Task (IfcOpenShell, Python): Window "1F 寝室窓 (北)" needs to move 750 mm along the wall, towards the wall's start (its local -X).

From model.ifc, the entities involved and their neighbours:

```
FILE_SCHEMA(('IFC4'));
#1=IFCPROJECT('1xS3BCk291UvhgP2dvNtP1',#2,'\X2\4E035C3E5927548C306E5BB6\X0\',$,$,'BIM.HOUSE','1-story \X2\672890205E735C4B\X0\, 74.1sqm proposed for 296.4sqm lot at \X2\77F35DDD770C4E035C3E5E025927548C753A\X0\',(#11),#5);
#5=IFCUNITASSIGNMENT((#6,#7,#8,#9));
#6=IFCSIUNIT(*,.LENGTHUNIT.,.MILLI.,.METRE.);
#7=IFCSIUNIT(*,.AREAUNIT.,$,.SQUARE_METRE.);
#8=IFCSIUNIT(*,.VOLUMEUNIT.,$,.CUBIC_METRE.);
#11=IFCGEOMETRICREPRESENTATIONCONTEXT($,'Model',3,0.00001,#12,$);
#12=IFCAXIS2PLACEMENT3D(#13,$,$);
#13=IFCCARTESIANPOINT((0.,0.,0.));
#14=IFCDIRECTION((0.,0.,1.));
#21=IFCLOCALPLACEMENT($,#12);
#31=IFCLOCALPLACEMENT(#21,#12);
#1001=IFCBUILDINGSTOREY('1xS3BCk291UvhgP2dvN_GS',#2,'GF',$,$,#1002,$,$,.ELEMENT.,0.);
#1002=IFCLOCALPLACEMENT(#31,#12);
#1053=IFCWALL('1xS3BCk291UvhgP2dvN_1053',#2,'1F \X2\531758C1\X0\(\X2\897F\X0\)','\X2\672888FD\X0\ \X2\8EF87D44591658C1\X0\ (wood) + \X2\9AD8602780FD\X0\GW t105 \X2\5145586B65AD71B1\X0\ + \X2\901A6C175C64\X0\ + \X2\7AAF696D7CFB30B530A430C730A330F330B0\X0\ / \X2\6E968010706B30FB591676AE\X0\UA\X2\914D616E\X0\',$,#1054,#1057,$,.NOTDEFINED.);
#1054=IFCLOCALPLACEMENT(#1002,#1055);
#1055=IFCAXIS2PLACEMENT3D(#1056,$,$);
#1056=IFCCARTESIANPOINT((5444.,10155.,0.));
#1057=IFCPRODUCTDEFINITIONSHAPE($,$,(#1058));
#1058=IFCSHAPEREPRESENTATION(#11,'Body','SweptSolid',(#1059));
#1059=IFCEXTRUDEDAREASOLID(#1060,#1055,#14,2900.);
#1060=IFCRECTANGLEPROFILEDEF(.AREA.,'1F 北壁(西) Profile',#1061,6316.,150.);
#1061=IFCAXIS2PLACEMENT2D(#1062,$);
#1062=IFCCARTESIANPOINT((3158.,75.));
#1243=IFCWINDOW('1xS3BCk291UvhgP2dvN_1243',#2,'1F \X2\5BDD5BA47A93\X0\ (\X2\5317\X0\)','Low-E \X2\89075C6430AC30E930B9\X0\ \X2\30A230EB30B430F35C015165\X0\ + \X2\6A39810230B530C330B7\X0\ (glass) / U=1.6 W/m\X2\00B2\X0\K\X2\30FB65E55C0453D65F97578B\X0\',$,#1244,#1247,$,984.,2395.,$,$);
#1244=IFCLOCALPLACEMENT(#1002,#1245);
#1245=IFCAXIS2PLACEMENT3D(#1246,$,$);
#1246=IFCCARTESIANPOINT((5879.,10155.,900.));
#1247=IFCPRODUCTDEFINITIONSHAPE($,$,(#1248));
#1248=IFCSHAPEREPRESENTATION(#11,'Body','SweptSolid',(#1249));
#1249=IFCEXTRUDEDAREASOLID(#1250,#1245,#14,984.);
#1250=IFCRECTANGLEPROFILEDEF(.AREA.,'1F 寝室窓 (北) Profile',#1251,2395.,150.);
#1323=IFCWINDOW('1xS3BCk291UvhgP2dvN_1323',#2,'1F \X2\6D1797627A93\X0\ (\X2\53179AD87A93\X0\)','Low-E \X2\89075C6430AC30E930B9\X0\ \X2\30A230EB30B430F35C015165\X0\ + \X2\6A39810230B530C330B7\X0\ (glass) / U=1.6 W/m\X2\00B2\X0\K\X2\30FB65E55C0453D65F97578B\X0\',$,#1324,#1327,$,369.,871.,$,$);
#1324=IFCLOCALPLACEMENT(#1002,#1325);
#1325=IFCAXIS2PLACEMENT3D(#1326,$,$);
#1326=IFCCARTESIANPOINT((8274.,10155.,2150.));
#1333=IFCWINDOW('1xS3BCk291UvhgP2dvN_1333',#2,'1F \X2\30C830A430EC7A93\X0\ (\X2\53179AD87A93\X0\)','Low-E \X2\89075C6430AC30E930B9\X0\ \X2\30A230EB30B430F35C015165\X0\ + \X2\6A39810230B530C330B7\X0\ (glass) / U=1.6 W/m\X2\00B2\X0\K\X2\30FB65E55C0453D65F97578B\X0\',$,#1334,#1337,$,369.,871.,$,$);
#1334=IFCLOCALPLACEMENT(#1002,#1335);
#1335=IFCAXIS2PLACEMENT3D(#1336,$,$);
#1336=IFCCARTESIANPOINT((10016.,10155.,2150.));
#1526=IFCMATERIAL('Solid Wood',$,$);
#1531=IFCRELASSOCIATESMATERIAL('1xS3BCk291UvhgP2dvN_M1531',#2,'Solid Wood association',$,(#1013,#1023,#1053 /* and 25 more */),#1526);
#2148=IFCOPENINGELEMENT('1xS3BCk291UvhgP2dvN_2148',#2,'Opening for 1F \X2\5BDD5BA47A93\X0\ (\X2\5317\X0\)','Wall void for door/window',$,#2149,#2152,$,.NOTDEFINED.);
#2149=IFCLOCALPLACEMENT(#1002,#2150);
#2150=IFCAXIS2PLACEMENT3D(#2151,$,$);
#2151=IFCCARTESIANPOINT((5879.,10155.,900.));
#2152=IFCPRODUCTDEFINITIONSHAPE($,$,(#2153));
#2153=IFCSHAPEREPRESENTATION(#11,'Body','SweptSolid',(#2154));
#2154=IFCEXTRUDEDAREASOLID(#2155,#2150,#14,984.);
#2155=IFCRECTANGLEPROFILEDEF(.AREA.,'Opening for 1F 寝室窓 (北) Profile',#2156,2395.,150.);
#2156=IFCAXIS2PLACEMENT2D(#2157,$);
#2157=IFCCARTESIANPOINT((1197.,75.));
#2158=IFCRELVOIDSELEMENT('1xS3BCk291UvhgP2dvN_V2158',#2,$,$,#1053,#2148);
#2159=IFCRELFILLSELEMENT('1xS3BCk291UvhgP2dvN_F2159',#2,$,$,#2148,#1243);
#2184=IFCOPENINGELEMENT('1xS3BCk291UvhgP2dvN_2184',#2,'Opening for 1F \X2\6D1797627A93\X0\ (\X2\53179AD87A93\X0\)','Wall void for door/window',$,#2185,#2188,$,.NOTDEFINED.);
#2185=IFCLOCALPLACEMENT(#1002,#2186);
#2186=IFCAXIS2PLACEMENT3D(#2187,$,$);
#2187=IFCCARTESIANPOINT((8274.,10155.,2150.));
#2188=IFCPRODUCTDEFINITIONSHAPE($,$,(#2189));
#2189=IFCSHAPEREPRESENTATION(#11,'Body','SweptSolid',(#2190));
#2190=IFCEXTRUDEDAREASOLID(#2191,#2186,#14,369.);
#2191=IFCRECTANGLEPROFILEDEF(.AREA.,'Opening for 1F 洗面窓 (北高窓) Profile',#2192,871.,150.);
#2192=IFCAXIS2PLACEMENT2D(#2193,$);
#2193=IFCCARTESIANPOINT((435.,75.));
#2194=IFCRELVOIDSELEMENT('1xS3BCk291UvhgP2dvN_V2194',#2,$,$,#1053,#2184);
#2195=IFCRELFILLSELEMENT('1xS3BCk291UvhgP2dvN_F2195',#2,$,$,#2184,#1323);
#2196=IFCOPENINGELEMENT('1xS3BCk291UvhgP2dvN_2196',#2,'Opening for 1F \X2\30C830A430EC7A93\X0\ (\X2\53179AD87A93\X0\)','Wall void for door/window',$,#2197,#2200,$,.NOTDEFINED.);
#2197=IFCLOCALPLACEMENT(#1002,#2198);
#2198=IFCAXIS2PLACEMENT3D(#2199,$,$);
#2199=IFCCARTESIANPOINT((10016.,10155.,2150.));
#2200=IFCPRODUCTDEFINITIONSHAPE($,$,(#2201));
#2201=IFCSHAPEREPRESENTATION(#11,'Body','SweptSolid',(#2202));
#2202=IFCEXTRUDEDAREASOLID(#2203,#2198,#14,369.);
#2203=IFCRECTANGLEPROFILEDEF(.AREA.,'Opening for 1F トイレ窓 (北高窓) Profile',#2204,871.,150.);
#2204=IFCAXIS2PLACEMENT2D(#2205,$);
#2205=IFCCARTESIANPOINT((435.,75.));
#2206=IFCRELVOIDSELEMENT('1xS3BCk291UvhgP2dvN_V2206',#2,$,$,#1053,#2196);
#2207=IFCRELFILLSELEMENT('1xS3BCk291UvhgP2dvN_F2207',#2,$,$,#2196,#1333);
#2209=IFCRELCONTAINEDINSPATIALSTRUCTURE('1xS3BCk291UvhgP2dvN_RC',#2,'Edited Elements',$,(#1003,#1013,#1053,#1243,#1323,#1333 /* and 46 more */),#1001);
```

```python
import ifcopenshell
import ifcopenshell.api.geometry
import ifcopenshell.util.placement
import ifcopenshell.util.unit

model = ifcopenshell.open("model.ifc")
unit_scale = ifcopenshell.util.unit.calculate_unit_scale(model)

window = model.by_guid("1xS3BCk291UvhgP2dvN_1243")
opening = window.FillsVoids[0].RelatingOpeningElement
wall = opening.VoidsElements[0].RelatingBuildingElement

wall_matrix = ifcopenshell.util.placement.get_local_placement(wall.ObjectPlacement)
shift = wall_matrix[:3, 0] * -0.75 / unit_scale
before = ifcopenshell.util.placement.get_local_placement(window.ObjectPlacement)[:3, 3].copy()

# The window is not placed relative to its opening, so move both.
for product in (opening, window):
    matrix = ifcopenshell.util.placement.get_local_placement(product.ObjectPlacement)
    matrix[:3, 3] += shift
    ifcopenshell.api.geometry.edit_object_placement(model, product=product, matrix=matrix, is_si=False)

after = ifcopenshell.util.placement.get_local_placement(window.ObjectPlacement)[:3, 3]
print("window moved by", (after - before).round(3) + 0.0)

model.write("model_v2.ifc")
```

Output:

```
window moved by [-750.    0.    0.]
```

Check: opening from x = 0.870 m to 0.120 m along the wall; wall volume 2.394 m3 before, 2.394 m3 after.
